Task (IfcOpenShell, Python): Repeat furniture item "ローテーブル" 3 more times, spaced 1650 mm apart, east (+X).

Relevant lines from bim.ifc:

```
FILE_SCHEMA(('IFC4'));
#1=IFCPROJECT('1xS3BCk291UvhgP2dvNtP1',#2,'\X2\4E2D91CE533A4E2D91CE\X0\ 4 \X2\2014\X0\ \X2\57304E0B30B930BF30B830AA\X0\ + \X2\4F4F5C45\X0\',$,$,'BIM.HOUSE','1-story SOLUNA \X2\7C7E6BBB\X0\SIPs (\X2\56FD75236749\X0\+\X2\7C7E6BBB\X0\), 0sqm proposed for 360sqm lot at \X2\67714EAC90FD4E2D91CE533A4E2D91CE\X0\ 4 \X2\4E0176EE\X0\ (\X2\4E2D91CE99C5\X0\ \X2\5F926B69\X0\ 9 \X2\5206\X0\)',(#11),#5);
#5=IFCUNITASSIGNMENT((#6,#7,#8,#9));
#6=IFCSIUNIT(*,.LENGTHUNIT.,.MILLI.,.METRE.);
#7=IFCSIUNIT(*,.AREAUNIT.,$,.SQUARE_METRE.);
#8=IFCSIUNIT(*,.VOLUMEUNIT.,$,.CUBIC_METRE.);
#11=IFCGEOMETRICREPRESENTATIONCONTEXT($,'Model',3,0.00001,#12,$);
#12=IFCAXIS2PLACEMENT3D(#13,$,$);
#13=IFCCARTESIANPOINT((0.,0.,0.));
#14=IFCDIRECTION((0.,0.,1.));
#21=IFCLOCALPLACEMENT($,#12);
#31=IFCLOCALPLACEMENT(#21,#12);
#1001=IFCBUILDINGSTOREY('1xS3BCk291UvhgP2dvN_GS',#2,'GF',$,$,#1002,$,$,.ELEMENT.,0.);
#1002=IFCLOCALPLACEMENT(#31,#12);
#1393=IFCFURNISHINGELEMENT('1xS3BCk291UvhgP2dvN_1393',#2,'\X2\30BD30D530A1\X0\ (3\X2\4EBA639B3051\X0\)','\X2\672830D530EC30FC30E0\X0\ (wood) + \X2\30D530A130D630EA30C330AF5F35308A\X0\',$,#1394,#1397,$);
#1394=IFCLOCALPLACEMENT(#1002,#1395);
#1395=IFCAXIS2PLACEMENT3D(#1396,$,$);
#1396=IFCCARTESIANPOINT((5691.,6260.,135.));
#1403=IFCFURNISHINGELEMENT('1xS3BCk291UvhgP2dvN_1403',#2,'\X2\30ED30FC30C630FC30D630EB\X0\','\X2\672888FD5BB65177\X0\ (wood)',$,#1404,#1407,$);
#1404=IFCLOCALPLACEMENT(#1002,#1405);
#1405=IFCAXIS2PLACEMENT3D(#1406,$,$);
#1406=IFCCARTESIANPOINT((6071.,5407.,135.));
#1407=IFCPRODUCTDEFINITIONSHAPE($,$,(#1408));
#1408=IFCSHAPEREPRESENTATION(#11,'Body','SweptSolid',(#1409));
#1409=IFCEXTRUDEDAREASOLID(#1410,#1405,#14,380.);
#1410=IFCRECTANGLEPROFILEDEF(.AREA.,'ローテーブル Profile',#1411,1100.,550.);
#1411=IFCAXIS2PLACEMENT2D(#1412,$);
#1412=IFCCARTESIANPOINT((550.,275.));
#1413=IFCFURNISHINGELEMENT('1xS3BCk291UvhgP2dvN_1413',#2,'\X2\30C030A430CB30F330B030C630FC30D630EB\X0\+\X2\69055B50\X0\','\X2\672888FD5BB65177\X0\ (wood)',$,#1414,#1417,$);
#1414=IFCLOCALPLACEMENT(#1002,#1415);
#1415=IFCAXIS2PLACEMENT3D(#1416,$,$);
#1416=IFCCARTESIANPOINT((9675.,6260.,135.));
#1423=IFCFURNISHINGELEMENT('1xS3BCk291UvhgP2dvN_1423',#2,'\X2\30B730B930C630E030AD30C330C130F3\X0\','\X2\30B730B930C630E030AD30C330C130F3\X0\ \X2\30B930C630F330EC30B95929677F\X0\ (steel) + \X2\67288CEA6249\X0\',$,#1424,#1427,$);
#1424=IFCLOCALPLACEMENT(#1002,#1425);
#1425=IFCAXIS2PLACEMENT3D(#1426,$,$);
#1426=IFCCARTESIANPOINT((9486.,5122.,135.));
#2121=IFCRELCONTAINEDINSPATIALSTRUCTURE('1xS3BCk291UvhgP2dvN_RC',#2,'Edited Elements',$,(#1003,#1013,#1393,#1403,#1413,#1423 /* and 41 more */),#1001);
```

```python
import numpy as np
import ifcopenshell
import ifcopenshell.api.geometry
import ifcopenshell.api.root
import ifcopenshell.util.element
import ifcopenshell.util.placement
import ifcopenshell.util.unit

model = ifcopenshell.open("bim.ifc")
unit_scale = ifcopenshell.util.unit.calculate_unit_scale(model)


def reuse_history(source, copy):
    """copy_class also copies each property set's owner history, people and application; keep the originals."""
    for rel in copy.IsDefinedBy:
        if rel.is_a("IfcRelDefinesByProperties") and (history := rel.RelatingPropertyDefinition.OwnerHistory):
            rel.RelatingPropertyDefinition.OwnerHistory = source.OwnerHistory
            ifcopenshell.util.element.remove_deep2(model, history)


source = model.by_id(1403)
base = ifcopenshell.util.placement.get_local_placement(source.ObjectPlacement)
step = np.array([1.0, 0.0, 0.0]) * 1.65 / unit_scale

for i in range(1, 4):
    copy = ifcopenshell.api.root.copy_class(model, product=source)
    copy.Representation = ifcopenshell.util.element.copy_deep(
        model, source.Representation, exclude=["IfcGeometricRepresentationContext", "IfcRepresentationMap"]
    )
    reuse_history(source, copy)
    matrix = base.copy()
    matrix[:3, 3] += i * step
    print("added at", matrix[:3, 3].round(3) + 0.0)
    ifcopenshell.api.geometry.edit_object_placement(model, product=copy, matrix=matrix, is_si=False)

model.write("bim_edited.ifc")
```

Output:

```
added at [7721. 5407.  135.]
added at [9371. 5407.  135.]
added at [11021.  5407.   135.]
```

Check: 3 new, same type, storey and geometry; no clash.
